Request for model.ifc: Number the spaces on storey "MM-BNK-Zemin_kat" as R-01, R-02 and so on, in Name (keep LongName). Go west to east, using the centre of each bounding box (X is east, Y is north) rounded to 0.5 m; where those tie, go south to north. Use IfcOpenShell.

First a look at what the model holds.

```python
import ifcopenshell
import ifcopenshell.util.element
import ifcopenshell.util.placement

model = ifcopenshell.open("model.ifc")
print(model.schema)
storey = next(s for s in model.by_type("IfcBuildingStorey") if s.Name == "MM-BNK-Zemin_kat")
spaces = [e for e in ifcopenshell.util.element.get_decomposition(storey) if e.is_a("IfcSpace")]
for e in sorted(spaces, key=lambda e: e.id()):
    origin = ifcopenshell.util.placement.get_local_placement(e.ObjectPlacement)[:3, 3]
    print(e.id(), e.Name, e.LongName, origin.round(2) + 0.0, sep=" | ")
```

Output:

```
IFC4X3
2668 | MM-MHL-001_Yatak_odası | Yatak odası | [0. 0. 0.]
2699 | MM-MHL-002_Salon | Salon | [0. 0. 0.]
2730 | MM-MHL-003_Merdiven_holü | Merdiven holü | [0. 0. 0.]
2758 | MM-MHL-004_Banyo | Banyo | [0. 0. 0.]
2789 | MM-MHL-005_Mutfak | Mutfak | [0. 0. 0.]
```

```python
import ifcopenshell
import ifcopenshell.geom
import ifcopenshell.util.element
import ifcopenshell.util.shape

model = ifcopenshell.open("model.ifc")
settings = ifcopenshell.geom.settings()
settings.set("use-world-coords", True)


def centre(element):
    shape = ifcopenshell.geom.create_shape(settings, element)
    return ifcopenshell.util.shape.get_bbox_centroid(shape.geometry)


storey = next(s for s in model.by_type("IfcBuildingStorey") if s.Name == "MM-BNK-Zemin_kat")
spaces = [e for e in ifcopenshell.util.element.get_decomposition(storey) if e.is_a("IfcSpace")]

# Insertion points can sit at a corner or the storey origin, so sort by the geometry (in metres).
centres = {e: centre(e) for e in spaces}
spaces.sort(key=lambda e: (round(centres[e][0] / 0.5), centres[e][1]))

for i, e in enumerate(spaces, start=1):
    number = f"R-{i:02d}"
    e.Name = number
    print(e.id(), number)

model.write("model_updated.ifc")
```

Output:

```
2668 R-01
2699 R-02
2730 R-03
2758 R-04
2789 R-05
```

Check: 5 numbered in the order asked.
